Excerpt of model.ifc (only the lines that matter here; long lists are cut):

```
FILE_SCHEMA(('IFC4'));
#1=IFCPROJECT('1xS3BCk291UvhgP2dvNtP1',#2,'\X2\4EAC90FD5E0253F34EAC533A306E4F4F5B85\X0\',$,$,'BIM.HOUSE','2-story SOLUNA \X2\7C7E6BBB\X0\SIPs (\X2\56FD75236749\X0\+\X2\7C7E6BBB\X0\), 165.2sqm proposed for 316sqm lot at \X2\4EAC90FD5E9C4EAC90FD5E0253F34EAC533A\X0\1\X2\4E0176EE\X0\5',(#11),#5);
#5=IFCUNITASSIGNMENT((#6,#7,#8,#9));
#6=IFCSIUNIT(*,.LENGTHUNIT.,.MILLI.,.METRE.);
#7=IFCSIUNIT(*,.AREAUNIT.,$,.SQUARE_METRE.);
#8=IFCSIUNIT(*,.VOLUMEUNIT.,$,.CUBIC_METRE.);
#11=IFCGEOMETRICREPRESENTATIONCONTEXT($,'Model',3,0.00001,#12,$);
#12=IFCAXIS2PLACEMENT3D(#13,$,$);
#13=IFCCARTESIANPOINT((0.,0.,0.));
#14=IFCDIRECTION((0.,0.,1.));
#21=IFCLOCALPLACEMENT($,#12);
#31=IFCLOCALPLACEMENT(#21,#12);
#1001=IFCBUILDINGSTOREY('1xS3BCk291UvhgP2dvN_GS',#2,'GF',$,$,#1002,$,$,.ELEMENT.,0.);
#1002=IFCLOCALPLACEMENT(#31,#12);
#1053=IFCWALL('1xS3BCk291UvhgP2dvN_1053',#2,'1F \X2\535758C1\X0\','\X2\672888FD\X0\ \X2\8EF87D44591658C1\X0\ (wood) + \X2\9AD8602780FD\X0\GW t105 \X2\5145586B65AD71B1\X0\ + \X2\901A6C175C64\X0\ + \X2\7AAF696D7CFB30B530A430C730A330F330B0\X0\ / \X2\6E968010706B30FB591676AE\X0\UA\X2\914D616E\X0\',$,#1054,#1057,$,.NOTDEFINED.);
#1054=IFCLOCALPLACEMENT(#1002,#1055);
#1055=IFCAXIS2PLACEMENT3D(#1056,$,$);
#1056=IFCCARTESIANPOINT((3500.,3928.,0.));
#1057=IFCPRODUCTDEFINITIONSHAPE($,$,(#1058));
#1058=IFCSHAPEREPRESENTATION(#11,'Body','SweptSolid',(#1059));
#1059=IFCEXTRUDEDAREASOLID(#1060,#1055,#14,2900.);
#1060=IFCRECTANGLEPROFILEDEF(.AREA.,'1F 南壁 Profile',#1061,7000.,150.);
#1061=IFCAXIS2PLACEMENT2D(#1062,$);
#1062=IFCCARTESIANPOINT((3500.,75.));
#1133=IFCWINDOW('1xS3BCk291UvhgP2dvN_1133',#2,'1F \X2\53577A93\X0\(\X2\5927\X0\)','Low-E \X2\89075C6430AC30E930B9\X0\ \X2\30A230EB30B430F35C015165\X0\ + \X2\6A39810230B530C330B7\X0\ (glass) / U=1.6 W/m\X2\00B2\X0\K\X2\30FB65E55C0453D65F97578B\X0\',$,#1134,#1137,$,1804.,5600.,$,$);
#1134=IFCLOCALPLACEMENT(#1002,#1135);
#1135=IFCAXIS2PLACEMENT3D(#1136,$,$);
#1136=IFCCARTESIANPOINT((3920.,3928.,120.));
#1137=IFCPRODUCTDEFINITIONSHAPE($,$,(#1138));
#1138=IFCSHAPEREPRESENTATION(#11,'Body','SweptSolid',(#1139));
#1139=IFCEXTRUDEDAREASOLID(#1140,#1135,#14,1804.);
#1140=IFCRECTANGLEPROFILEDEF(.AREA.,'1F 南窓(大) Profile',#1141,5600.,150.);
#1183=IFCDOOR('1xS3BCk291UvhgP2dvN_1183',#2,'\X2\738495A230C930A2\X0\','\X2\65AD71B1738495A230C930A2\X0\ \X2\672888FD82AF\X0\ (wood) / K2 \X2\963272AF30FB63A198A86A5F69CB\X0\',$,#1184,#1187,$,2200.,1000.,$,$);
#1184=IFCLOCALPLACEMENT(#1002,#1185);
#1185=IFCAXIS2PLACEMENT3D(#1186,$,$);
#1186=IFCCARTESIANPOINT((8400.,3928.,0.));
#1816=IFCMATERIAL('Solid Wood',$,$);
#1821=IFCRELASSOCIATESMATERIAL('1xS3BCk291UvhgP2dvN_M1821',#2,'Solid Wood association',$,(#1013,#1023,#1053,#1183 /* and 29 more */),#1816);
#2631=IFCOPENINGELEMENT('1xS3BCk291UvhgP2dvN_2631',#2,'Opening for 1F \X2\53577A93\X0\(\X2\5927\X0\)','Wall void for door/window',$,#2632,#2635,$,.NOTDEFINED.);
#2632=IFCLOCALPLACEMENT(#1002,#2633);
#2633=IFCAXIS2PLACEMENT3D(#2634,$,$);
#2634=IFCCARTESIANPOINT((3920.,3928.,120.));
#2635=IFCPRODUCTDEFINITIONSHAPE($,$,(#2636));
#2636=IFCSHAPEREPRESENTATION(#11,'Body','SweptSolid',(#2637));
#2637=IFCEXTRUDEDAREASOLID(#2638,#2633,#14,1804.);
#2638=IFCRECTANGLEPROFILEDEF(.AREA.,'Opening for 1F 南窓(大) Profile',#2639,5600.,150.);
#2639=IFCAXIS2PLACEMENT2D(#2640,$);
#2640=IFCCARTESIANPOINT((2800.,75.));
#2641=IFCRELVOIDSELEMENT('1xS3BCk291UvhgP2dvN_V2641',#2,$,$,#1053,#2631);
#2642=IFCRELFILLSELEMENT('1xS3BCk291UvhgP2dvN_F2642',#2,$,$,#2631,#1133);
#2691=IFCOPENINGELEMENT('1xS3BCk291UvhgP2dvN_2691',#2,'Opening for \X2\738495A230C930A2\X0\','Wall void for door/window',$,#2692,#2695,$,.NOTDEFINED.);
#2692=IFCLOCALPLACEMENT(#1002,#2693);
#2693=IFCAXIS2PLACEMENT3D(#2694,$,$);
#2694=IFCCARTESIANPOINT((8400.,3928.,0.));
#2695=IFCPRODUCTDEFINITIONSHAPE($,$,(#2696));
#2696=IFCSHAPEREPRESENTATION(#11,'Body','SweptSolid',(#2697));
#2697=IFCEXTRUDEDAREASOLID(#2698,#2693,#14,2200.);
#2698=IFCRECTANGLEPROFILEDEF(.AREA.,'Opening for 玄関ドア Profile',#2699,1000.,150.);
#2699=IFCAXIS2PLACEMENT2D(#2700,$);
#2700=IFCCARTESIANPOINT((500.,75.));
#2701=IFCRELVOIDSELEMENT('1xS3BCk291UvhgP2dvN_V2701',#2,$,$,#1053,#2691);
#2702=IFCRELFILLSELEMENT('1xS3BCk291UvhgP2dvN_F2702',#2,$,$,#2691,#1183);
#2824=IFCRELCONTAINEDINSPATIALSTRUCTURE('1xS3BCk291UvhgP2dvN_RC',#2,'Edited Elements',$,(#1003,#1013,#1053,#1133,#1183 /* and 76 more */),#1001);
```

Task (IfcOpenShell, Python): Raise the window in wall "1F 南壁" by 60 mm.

```python
import numpy as np
import ifcopenshell
import ifcopenshell.api.geometry
import ifcopenshell.util.placement
import ifcopenshell.util.unit

model = ifcopenshell.open("model.ifc")
unit_scale = ifcopenshell.util.unit.calculate_unit_scale(model)

window = model.by_guid("1xS3BCk291UvhgP2dvN_1133")
opening = window.FillsVoids[0].RelatingOpeningElement
dz = 60.0

shift = np.array([0.0, 0.0, dz])
# The window is not placed relative to its opening, so move both.
for product in (opening, window):
    matrix = ifcopenshell.util.placement.get_local_placement(product.ObjectPlacement)
    matrix[:3, 3] += shift
    ifcopenshell.api.geometry.edit_object_placement(model, product=product, matrix=matrix, is_si=False)

print(f"moved by {dz * unit_scale:+.3f} m")

model.write("model_rev.ifc")
```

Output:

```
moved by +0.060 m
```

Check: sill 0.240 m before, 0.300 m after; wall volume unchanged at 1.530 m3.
